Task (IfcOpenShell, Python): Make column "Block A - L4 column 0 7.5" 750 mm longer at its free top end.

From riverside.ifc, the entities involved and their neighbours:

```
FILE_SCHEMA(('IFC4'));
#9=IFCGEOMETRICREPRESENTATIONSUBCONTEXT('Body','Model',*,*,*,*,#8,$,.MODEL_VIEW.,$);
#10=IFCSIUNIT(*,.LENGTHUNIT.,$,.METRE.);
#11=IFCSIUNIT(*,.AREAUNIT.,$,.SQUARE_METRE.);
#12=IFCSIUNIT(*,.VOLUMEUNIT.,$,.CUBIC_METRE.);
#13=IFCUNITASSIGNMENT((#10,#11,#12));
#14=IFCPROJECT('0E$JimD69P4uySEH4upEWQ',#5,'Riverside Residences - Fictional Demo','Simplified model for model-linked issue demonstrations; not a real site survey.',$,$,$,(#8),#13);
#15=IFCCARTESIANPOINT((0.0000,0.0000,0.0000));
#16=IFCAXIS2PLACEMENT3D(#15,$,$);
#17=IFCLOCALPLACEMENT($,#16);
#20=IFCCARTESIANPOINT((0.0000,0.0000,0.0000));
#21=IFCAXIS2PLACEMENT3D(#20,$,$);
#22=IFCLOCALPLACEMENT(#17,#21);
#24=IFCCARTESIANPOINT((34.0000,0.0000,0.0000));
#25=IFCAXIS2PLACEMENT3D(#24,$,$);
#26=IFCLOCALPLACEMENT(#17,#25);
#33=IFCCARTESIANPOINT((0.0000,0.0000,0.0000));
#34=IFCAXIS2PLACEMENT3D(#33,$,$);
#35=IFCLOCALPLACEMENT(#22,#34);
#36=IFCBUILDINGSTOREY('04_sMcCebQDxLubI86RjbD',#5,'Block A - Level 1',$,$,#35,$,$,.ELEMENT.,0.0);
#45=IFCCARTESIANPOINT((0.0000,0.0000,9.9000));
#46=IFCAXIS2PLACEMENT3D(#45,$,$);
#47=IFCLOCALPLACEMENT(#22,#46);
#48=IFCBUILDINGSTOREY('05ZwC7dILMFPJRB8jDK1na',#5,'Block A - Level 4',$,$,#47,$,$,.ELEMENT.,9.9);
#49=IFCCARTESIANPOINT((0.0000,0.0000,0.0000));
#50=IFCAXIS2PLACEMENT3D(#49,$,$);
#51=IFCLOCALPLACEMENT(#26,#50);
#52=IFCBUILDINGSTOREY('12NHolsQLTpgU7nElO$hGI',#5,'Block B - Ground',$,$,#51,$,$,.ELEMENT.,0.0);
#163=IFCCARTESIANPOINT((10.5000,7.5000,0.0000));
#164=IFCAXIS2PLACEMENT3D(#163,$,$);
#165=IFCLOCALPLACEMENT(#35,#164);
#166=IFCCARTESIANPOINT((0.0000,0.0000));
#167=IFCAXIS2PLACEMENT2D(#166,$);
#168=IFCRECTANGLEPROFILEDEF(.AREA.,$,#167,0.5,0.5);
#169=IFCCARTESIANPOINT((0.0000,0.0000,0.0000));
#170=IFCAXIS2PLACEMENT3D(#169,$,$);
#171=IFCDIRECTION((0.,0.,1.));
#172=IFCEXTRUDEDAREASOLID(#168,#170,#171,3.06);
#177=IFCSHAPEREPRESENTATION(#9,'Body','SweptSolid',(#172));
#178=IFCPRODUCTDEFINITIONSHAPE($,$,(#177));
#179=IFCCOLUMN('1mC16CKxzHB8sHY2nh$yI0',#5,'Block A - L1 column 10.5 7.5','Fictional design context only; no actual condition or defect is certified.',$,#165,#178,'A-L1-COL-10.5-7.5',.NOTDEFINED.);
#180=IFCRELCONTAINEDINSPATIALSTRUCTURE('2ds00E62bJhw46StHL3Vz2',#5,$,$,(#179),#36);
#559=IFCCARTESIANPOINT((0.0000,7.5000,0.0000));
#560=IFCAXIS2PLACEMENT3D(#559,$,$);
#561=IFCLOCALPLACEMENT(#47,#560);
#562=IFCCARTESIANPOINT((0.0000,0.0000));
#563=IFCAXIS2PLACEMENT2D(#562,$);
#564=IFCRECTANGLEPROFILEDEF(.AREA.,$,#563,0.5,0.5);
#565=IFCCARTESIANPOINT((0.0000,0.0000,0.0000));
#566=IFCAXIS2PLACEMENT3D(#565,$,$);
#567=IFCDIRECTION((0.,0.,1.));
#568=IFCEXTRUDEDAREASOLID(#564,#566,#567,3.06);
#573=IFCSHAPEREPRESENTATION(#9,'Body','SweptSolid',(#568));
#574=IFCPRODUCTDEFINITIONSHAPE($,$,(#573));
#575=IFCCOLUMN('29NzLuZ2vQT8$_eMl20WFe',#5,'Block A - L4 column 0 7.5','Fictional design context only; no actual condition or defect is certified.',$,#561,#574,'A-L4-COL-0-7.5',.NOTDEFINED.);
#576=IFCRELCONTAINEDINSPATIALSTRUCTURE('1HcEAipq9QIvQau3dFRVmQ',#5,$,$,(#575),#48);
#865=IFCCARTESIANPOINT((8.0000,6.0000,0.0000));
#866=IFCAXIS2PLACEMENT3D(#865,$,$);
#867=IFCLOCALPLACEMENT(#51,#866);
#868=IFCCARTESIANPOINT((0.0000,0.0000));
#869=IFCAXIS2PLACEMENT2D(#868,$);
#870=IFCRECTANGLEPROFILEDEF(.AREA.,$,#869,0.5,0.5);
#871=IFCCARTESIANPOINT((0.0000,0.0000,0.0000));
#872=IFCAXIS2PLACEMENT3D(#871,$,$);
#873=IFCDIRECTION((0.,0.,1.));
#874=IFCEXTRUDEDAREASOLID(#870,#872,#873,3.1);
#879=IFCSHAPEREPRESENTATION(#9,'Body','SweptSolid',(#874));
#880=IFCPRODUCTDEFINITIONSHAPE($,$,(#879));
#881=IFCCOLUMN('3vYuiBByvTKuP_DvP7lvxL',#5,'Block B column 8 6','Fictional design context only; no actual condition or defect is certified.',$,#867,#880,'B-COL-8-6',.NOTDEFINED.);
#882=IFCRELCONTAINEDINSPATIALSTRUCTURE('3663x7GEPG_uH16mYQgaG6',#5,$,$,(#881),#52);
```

```python
import ifcopenshell
import ifcopenshell.util.representation
import ifcopenshell.util.unit

model = ifcopenshell.open("riverside.ifc")
unit_scale = ifcopenshell.util.unit.calculate_unit_scale(model)

member = model.by_guid("29NzLuZ2vQT8$_eMl20WFe")
change = 0.75 / unit_scale

# The extrusion runs towards the end named, so only its depth changes.
body = ifcopenshell.util.representation.get_representation(member, "Model", "Body")
solid = body.Items[0]
old_length = solid.Depth
solid.Depth += change

print(f"length {old_length:g} -> {solid.Depth:g}")

model.write("riverside-out.ifc")
```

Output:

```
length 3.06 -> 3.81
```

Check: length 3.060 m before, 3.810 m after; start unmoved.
